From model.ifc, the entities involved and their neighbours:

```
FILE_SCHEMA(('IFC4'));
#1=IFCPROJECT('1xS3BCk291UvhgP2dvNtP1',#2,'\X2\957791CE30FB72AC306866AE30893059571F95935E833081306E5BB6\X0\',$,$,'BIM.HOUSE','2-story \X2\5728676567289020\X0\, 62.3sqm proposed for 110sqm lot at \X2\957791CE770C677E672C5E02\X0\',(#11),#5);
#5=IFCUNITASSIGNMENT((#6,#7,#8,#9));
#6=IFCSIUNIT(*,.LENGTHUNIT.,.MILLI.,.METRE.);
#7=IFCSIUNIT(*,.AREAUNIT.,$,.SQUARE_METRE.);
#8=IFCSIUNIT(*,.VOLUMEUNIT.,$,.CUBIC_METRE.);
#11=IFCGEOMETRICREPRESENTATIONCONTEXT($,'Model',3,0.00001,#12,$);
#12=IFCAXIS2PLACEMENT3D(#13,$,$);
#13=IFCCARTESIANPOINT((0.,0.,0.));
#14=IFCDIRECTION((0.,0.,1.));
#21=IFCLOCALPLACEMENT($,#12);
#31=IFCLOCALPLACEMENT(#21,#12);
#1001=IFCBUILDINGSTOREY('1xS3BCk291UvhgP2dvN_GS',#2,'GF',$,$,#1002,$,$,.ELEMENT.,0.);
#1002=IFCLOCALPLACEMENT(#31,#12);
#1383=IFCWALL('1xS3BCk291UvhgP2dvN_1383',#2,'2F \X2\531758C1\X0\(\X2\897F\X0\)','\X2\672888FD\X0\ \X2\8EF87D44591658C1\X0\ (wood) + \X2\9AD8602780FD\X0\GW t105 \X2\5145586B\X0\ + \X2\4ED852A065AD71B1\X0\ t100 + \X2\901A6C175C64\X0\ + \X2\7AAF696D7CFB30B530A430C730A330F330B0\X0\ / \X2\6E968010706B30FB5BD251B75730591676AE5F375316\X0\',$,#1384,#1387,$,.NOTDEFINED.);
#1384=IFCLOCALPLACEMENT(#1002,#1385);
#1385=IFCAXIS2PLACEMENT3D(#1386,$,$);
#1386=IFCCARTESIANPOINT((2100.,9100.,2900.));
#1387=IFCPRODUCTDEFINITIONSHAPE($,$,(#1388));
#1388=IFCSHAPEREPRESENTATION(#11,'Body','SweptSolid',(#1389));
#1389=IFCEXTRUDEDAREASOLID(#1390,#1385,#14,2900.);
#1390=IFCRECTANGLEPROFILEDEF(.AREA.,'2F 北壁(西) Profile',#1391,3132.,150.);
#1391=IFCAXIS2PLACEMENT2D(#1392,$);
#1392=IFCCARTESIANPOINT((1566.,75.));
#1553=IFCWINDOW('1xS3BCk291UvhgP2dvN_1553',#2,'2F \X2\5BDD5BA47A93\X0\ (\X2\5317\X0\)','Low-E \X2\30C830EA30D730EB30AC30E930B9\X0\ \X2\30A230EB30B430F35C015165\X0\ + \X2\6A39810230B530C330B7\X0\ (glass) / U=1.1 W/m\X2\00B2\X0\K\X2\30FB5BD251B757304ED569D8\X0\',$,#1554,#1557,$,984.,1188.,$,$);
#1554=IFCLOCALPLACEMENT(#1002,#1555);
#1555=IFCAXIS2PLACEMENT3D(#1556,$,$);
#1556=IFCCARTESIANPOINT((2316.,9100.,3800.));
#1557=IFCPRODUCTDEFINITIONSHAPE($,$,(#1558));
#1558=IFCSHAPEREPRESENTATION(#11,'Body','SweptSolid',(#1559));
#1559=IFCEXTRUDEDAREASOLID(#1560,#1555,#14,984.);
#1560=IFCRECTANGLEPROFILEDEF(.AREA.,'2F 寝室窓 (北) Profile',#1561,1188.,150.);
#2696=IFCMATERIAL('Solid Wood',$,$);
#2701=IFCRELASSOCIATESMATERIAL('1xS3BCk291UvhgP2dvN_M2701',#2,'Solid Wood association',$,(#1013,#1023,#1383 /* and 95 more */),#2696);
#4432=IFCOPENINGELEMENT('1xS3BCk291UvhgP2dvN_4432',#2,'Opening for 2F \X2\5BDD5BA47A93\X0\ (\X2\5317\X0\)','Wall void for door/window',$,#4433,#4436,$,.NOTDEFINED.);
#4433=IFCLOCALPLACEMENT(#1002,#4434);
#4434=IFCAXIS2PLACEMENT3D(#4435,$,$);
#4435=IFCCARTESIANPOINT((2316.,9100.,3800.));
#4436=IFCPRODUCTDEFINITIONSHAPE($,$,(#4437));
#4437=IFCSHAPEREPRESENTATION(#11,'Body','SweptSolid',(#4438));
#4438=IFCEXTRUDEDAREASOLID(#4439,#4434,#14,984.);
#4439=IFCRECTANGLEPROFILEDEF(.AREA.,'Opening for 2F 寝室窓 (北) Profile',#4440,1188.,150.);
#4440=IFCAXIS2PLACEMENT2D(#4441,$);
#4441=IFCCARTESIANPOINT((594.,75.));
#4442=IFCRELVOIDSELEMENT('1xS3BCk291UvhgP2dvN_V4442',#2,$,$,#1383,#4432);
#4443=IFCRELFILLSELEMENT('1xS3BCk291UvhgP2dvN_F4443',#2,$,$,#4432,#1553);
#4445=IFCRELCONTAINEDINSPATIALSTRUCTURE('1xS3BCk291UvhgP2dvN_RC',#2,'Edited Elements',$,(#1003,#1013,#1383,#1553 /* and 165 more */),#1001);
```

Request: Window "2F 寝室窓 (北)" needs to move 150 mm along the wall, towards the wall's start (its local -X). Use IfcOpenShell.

```python
import ifcopenshell
import ifcopenshell.api.geometry
import ifcopenshell.util.placement
import ifcopenshell.util.unit

model = ifcopenshell.open("model.ifc")
unit_scale = ifcopenshell.util.unit.calculate_unit_scale(model)

window = model.by_guid("1xS3BCk291UvhgP2dvN_1553")
opening = window.FillsVoids[0].RelatingOpeningElement
wall = opening.VoidsElements[0].RelatingBuildingElement

wall_matrix = ifcopenshell.util.placement.get_local_placement(wall.ObjectPlacement)
shift = wall_matrix[:3, 0] * -0.15 / unit_scale
before = ifcopenshell.util.placement.get_local_placement(window.ObjectPlacement)[:3, 3].copy()

# The window is not placed relative to its opening, so move both.
for product in (opening, window):
    matrix = ifcopenshell.util.placement.get_local_placement(product.ObjectPlacement)
    matrix[:3, 3] += shift
    ifcopenshell.api.geometry.edit_object_placement(model, product=product, matrix=matrix, is_si=False)

after = ifcopenshell.util.placement.get_local_placement(window.ObjectPlacement)[:3, 3]
print("window moved by", (after - before).round(3) + 0.0)

model.write("model_edited.ifc")
```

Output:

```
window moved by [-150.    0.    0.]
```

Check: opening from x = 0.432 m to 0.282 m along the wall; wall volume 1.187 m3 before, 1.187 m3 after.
